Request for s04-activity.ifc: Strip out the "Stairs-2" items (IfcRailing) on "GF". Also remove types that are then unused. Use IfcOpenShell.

First a look at what the model holds.

```python
import ifcopenshell
import ifcopenshell.util.element

model = ifcopenshell.open("s04-activity.ifc")
print(model.schema)
storey = next(s for s in model.by_type("IfcBuildingStorey") if s.Name == "GF")
railings = [e for e in ifcopenshell.util.element.get_decomposition(storey) if e.is_a("IfcRailing")]
seen = {}
for e in railings:
    element_type = ifcopenshell.util.element.get_type(e)
    name = element_type.Name if element_type not in (None, e) else None
    seen[name] = seen.get(name, 0) + 1
for name, count in sorted(seen.items(), key=str):
    print(count, "x", name)
```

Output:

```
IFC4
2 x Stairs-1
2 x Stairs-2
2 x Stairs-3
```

```python
import ifcopenshell
import ifcopenshell.api.root
import ifcopenshell.util.element

model = ifcopenshell.open("s04-activity.ifc")

storey = next(s for s in model.by_type("IfcBuildingStorey") if s.Name == "GF")
railings = [e for e in ifcopenshell.util.element.get_decomposition(storey) if e.is_a("IfcRailing")]
targets = [e for e in railings if (t := ifcopenshell.util.element.get_type(e)) not in (None, e) and t.Name == "Stairs-2"]
types = {ifcopenshell.util.element.get_type(e) for e in targets} - {None, *targets}

for e in targets:
    ifcopenshell.api.root.remove_product(model, product=e)
print(len(targets), "removed")

unused = [t for t in types if not ifcopenshell.util.element.get_types(t)]
for t in unused:
    ifcopenshell.api.root.remove_product(model, product=t)
print(len(unused), "unused types removed")

model.write("s04-activity_edited.ifc")
```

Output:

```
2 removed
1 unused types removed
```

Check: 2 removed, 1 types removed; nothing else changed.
